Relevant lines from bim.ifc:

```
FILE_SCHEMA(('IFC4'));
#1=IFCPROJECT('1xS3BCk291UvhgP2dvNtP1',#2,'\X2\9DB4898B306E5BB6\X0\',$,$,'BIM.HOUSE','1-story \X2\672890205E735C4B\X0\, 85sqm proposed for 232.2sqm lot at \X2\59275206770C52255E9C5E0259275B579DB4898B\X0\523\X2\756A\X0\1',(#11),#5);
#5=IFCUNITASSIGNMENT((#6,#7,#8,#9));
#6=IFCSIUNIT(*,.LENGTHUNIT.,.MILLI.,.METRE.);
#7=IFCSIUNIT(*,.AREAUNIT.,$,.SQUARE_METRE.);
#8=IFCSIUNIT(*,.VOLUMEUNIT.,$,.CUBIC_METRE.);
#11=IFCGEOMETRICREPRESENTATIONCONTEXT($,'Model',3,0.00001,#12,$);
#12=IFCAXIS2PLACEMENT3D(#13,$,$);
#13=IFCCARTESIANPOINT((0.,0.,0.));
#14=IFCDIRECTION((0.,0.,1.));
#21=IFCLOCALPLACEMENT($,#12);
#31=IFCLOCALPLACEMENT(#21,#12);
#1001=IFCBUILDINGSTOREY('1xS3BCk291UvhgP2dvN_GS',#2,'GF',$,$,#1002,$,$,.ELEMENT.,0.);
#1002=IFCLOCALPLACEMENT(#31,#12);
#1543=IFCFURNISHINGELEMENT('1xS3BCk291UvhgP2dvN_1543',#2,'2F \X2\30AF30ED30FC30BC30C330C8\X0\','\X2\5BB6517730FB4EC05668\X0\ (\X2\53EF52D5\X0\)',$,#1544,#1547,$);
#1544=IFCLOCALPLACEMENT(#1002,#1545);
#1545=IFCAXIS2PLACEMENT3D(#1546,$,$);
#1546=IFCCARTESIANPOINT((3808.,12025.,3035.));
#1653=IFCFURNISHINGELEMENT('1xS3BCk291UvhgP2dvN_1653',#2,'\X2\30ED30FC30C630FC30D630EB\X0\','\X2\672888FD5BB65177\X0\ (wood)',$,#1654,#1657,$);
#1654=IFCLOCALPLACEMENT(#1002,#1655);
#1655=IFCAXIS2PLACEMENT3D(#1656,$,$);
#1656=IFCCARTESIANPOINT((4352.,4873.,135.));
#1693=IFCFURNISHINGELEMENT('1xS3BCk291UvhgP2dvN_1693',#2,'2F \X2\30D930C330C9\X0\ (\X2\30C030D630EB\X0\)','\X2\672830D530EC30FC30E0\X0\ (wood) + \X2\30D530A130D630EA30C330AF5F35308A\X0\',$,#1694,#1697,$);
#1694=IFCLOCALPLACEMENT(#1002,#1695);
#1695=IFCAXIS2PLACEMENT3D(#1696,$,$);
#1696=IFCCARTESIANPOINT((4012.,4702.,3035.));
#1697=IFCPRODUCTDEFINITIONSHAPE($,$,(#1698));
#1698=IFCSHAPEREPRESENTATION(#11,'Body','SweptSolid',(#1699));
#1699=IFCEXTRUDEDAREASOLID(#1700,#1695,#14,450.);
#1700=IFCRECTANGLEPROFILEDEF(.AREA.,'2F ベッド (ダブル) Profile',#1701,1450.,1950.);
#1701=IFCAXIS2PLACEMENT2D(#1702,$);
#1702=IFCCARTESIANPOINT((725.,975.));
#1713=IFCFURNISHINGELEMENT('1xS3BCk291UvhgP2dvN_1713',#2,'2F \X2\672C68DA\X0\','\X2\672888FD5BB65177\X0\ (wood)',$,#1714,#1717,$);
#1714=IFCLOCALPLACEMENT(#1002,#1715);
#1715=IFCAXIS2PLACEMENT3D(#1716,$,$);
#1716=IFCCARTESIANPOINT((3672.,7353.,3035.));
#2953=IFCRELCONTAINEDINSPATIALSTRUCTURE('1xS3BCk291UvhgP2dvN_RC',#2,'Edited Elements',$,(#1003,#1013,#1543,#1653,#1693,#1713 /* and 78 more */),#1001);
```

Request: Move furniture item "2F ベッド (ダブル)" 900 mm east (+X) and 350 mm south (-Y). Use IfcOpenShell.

```python
import ifcopenshell
import ifcopenshell.api.geometry
import ifcopenshell.util.placement

model = ifcopenshell.open("bim.ifc")

item = model.by_guid("1xS3BCk291UvhgP2dvN_1693")
matrix = ifcopenshell.util.placement.get_local_placement(item.ObjectPlacement)
matrix[0, 3] += 900.0
matrix[1, 3] -= 350.0
ifcopenshell.api.geometry.edit_object_placement(model, product=item, matrix=matrix, is_si=False)

print(ifcopenshell.util.placement.get_local_placement(item.ObjectPlacement).round(3) + 0.0)

model.write("bim_v2.ifc")
```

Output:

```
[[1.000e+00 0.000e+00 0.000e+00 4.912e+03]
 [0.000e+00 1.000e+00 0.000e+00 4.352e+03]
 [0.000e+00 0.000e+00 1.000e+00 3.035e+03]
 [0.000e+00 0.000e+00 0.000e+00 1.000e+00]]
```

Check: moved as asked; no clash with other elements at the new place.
